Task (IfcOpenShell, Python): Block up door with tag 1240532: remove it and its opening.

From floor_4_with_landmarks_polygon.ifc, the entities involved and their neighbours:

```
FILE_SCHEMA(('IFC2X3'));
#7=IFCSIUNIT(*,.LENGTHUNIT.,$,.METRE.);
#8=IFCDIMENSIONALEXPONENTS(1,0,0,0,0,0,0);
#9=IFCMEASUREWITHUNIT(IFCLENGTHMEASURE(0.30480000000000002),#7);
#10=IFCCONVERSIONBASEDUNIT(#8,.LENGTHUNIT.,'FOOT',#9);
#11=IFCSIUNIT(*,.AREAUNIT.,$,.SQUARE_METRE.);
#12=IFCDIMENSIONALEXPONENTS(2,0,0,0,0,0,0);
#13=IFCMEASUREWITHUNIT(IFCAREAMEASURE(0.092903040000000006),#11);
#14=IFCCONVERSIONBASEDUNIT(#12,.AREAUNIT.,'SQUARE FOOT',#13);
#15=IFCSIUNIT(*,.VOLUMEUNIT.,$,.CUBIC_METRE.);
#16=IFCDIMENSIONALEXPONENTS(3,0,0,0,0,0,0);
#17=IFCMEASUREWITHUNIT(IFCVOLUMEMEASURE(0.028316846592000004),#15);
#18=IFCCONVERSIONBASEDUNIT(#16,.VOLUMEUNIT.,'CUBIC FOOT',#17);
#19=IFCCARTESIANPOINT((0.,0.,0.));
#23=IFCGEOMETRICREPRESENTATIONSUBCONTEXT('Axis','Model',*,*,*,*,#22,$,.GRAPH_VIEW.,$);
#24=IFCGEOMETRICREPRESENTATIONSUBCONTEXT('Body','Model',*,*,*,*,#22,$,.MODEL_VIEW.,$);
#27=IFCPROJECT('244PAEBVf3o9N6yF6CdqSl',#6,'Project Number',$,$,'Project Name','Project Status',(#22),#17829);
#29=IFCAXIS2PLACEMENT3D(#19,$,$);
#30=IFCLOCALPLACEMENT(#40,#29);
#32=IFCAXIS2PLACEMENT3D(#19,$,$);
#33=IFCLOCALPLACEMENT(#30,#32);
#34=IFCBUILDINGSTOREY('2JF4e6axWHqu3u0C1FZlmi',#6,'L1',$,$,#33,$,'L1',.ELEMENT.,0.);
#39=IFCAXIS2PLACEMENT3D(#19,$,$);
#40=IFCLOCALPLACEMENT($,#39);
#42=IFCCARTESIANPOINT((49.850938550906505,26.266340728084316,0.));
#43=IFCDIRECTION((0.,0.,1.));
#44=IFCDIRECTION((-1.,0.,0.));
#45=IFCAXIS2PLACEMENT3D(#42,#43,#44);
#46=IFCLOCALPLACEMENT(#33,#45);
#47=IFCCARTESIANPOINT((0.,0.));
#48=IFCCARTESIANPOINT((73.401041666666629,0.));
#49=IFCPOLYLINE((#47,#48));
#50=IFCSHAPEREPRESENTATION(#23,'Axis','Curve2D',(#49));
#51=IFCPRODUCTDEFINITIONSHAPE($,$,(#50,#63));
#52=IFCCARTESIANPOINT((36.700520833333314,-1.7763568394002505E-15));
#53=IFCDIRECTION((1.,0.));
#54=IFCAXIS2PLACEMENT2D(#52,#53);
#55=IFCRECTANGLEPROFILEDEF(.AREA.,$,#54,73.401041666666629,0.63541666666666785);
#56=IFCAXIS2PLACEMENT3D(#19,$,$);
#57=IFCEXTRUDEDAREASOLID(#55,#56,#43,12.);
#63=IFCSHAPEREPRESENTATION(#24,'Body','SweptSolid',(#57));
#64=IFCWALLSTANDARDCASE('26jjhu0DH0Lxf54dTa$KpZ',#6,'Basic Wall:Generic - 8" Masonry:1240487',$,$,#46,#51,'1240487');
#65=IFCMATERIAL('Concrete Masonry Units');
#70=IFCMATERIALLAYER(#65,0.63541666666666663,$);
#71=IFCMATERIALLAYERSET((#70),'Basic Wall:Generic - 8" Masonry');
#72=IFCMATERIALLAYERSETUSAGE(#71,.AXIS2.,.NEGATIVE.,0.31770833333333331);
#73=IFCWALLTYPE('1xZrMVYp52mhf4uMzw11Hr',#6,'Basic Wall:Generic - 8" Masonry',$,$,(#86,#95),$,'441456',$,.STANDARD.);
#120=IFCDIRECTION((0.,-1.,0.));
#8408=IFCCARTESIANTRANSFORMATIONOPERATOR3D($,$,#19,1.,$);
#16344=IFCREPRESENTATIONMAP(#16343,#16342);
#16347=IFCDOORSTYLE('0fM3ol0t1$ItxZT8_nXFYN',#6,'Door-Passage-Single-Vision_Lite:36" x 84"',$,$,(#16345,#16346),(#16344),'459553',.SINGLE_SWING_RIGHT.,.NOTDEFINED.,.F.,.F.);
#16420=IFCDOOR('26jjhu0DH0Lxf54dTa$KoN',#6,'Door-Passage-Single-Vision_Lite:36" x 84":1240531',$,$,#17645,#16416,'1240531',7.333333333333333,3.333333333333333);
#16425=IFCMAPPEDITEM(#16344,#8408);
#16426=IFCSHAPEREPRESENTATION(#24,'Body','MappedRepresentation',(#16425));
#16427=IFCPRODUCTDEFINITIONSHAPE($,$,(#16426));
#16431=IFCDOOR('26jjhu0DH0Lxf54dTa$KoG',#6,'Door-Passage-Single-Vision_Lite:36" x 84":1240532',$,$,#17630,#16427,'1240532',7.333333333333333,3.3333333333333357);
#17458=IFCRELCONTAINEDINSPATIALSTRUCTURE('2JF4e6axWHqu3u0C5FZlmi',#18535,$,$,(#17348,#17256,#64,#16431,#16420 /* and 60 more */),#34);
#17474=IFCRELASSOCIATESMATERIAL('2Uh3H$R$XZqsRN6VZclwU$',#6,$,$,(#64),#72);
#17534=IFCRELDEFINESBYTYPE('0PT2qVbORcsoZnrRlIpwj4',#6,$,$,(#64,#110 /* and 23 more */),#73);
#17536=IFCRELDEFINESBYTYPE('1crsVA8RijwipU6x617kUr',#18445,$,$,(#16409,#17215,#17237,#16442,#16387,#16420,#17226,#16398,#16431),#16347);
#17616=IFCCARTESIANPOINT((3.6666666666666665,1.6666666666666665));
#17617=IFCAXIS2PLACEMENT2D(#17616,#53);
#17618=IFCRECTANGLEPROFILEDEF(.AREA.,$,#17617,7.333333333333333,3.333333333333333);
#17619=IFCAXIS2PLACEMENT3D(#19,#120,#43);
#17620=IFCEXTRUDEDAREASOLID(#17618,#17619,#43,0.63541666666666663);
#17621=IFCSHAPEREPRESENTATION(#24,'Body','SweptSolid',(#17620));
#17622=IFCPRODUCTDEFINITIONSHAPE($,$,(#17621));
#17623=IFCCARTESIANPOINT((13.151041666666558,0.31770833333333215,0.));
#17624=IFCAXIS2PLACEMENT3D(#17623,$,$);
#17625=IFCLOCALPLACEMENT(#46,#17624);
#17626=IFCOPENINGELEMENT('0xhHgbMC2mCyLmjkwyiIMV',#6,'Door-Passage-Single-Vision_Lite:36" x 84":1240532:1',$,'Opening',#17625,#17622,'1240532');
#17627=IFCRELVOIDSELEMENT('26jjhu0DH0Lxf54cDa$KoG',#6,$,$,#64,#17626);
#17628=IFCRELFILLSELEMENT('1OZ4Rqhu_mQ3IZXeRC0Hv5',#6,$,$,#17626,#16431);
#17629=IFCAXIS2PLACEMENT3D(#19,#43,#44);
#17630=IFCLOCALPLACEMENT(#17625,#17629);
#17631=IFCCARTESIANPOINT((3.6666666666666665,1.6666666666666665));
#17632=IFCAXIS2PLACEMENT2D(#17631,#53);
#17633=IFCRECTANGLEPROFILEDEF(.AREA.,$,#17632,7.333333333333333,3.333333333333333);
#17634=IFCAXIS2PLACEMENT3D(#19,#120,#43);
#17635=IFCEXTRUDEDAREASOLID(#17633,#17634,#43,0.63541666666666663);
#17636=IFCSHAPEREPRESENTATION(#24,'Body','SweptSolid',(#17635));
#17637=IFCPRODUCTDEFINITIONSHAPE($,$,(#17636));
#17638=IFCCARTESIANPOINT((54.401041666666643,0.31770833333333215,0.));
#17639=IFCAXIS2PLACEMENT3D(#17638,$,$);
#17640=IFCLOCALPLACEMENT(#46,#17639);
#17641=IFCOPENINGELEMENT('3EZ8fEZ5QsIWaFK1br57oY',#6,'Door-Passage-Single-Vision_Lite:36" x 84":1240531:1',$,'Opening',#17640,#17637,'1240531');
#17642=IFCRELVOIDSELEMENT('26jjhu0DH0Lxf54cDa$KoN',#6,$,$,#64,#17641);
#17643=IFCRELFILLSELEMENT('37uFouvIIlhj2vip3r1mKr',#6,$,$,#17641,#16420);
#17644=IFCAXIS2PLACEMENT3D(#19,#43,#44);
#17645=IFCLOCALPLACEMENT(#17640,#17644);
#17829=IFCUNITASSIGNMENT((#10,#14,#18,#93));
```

```python
import ifcopenshell
import ifcopenshell.api.feature
import ifcopenshell.api.root
import ifcopenshell.geom
import ifcopenshell.util.shape

model = ifcopenshell.open("floor_4_with_landmarks_polygon.ifc")
settings = ifcopenshell.geom.settings()


def volume(element):
    """Net volume in cubic metres, openings subtracted."""
    shape = ifcopenshell.geom.create_shape(settings, element)
    return ifcopenshell.util.shape.get_volume(shape.geometry)


door = model.by_guid("26jjhu0DH0Lxf54dTa$KoG")
opening = door.FillsVoids[0].RelatingOpeningElement
wall = opening.VoidsElements[0].RelatingBuildingElement
before = volume(wall)

ifcopenshell.api.root.remove_product(model, product=door)
ifcopenshell.api.feature.remove_feature(model, feature=opening)

after = volume(wall)

print(f"wall volume {before:.3f} -> {after:.3f} m3")

model.write("floor_4_with_landmarks_polygon-out.ifc")
```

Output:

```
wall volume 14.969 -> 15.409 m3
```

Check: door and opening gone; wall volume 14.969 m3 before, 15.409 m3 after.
